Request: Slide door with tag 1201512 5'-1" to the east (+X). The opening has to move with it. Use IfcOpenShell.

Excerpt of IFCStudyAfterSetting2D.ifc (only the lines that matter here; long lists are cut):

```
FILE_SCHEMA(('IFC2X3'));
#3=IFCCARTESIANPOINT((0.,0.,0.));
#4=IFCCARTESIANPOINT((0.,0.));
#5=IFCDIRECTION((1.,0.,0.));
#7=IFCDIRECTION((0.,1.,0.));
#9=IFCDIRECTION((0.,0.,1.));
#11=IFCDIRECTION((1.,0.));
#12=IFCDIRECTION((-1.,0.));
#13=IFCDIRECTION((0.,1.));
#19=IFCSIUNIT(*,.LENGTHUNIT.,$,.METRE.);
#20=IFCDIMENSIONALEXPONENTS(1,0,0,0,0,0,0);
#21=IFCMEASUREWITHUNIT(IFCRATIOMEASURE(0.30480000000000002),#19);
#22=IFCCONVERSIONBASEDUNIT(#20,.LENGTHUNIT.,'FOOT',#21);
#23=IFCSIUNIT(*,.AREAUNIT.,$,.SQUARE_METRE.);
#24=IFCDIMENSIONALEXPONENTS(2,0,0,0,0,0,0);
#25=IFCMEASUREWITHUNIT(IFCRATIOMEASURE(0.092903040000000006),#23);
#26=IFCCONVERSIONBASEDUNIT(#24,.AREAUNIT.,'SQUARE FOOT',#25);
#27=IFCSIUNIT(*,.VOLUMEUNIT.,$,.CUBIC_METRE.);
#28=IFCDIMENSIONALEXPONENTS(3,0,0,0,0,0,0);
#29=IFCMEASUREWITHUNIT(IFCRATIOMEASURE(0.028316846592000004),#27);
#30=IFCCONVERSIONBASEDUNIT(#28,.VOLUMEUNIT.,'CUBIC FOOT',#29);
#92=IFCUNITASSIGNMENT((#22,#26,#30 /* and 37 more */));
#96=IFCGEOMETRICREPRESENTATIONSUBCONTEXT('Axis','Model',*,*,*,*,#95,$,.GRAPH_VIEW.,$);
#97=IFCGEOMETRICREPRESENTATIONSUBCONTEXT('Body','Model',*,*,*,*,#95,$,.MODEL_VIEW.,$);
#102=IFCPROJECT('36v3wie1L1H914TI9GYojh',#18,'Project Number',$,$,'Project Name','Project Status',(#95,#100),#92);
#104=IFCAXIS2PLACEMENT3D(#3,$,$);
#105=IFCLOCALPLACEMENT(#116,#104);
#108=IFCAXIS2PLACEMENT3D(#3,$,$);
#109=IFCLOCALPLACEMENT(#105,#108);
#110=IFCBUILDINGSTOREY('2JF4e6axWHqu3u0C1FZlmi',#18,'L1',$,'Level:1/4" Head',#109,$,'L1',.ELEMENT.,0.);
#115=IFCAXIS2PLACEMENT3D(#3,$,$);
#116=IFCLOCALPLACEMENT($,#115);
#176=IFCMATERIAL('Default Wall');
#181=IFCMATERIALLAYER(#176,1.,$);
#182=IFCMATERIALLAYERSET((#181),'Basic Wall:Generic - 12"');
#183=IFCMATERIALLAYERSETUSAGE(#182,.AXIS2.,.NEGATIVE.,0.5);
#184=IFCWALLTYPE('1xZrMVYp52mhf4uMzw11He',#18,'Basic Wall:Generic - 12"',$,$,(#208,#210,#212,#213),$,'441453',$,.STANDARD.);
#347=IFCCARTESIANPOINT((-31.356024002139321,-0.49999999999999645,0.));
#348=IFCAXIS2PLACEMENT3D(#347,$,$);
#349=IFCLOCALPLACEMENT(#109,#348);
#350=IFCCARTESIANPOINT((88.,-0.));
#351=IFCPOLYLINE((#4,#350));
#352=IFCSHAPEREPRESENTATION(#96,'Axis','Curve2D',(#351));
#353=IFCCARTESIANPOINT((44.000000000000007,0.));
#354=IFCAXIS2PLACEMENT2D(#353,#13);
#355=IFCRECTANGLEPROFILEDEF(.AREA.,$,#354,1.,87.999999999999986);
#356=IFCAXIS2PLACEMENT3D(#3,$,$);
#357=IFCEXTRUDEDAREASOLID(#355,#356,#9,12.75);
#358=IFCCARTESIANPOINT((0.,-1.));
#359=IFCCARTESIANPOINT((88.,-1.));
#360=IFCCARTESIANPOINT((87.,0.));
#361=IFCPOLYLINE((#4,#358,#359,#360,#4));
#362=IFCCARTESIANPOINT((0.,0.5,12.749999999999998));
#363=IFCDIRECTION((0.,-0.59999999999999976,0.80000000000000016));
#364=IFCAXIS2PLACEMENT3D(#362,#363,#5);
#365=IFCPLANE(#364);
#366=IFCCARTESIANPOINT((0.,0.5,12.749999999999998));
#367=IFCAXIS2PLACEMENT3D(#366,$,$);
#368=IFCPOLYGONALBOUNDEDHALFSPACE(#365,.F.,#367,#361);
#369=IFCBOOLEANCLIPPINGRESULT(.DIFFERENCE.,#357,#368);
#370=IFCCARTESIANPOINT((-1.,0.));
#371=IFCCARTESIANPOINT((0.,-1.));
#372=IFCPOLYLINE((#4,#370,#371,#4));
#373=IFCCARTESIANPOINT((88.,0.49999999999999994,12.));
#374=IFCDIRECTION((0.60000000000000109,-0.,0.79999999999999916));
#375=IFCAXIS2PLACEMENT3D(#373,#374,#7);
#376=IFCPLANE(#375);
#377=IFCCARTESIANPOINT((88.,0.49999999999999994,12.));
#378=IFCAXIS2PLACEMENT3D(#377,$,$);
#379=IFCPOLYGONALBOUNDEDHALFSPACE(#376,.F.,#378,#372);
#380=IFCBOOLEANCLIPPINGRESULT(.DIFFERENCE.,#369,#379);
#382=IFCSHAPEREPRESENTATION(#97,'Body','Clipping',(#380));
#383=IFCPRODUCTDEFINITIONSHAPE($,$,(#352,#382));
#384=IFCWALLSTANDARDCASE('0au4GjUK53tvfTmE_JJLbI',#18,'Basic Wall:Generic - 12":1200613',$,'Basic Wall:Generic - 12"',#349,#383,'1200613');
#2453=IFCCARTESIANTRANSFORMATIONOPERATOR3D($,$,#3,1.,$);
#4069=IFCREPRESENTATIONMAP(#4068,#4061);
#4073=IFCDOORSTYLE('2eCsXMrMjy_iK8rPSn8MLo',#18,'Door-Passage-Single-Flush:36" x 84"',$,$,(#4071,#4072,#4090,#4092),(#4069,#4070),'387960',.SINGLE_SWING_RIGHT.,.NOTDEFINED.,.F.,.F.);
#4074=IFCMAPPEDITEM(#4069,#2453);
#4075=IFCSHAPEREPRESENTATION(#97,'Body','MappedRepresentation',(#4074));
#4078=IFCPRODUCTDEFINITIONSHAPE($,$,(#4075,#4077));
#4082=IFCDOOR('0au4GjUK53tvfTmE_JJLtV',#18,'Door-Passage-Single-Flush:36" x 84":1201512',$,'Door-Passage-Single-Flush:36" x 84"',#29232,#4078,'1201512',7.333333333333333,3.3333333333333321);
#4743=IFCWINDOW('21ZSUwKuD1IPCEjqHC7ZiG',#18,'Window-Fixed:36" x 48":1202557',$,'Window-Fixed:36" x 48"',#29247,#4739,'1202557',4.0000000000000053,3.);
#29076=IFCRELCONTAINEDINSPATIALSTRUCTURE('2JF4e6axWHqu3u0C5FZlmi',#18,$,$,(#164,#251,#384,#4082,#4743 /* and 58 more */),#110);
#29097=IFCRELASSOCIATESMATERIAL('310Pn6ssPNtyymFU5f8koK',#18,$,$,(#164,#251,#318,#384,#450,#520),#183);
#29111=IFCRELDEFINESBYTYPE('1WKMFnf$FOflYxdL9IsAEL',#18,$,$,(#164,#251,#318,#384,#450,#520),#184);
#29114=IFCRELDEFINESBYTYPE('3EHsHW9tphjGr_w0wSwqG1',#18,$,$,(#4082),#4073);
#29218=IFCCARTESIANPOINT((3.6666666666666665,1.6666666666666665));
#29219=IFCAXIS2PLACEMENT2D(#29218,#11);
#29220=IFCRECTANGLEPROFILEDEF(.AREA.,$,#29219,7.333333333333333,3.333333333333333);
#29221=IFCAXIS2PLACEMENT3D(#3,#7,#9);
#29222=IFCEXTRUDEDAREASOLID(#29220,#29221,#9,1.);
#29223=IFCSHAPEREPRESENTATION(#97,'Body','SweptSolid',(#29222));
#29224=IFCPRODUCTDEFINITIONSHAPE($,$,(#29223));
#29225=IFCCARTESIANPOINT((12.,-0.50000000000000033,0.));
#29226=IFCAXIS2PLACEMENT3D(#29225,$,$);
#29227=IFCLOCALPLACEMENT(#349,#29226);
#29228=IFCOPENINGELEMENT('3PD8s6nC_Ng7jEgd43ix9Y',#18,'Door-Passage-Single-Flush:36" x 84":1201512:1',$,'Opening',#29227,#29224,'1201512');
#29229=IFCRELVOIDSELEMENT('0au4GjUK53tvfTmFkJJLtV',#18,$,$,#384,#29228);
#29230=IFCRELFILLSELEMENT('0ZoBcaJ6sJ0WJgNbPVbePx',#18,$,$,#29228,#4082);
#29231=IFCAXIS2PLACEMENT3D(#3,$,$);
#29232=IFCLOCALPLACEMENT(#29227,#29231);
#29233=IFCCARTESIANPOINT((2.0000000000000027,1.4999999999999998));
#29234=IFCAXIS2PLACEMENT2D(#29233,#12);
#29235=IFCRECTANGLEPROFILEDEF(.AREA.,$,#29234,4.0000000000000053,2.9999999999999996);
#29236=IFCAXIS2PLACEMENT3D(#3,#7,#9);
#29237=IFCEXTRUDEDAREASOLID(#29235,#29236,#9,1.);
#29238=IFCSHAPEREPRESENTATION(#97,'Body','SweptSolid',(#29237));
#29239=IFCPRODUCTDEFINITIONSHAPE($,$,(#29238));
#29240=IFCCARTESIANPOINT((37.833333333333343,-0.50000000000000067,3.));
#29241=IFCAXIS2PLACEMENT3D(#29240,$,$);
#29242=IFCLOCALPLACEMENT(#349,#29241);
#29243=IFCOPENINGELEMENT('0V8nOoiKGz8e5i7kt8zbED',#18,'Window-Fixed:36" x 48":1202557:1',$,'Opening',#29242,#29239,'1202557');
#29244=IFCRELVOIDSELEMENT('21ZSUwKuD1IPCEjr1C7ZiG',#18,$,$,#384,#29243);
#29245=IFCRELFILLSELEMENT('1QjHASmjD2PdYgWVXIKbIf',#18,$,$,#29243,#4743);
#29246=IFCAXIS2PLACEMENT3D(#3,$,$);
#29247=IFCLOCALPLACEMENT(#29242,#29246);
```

```python
import ifcopenshell
import ifcopenshell.api.geometry
import ifcopenshell.util.placement
import ifcopenshell.util.unit

model = ifcopenshell.open("IFCStudyAfterSetting2D.ifc")
unit_scale = ifcopenshell.util.unit.calculate_unit_scale(model)

door = model.by_id(4082)
opening = door.FillsVoids[0].RelatingOpeningElement
wall = opening.VoidsElements[0].RelatingBuildingElement

wall_matrix = ifcopenshell.util.placement.get_local_placement(wall.ObjectPlacement)
shift = wall_matrix[:3, 0] * 61 * 0.0254 / unit_scale
before = ifcopenshell.util.placement.get_local_placement(door.ObjectPlacement)[:3, 3].copy()

# The door is placed relative to its opening, so it follows when the opening moves.
matrix = ifcopenshell.util.placement.get_local_placement(opening.ObjectPlacement)
matrix[:3, 3] += shift
ifcopenshell.api.geometry.edit_object_placement(
    model, product=opening, matrix=matrix, is_si=False, should_transform_children=True
)

after = ifcopenshell.util.placement.get_local_placement(door.ObjectPlacement)[:3, 3]
print("door moved by", (after - before).round(3) + 0.0)

model.write("IFCStudyAfterSetting2D_edited.ifc")
```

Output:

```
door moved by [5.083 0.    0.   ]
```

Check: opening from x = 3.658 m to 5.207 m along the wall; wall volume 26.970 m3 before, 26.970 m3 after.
